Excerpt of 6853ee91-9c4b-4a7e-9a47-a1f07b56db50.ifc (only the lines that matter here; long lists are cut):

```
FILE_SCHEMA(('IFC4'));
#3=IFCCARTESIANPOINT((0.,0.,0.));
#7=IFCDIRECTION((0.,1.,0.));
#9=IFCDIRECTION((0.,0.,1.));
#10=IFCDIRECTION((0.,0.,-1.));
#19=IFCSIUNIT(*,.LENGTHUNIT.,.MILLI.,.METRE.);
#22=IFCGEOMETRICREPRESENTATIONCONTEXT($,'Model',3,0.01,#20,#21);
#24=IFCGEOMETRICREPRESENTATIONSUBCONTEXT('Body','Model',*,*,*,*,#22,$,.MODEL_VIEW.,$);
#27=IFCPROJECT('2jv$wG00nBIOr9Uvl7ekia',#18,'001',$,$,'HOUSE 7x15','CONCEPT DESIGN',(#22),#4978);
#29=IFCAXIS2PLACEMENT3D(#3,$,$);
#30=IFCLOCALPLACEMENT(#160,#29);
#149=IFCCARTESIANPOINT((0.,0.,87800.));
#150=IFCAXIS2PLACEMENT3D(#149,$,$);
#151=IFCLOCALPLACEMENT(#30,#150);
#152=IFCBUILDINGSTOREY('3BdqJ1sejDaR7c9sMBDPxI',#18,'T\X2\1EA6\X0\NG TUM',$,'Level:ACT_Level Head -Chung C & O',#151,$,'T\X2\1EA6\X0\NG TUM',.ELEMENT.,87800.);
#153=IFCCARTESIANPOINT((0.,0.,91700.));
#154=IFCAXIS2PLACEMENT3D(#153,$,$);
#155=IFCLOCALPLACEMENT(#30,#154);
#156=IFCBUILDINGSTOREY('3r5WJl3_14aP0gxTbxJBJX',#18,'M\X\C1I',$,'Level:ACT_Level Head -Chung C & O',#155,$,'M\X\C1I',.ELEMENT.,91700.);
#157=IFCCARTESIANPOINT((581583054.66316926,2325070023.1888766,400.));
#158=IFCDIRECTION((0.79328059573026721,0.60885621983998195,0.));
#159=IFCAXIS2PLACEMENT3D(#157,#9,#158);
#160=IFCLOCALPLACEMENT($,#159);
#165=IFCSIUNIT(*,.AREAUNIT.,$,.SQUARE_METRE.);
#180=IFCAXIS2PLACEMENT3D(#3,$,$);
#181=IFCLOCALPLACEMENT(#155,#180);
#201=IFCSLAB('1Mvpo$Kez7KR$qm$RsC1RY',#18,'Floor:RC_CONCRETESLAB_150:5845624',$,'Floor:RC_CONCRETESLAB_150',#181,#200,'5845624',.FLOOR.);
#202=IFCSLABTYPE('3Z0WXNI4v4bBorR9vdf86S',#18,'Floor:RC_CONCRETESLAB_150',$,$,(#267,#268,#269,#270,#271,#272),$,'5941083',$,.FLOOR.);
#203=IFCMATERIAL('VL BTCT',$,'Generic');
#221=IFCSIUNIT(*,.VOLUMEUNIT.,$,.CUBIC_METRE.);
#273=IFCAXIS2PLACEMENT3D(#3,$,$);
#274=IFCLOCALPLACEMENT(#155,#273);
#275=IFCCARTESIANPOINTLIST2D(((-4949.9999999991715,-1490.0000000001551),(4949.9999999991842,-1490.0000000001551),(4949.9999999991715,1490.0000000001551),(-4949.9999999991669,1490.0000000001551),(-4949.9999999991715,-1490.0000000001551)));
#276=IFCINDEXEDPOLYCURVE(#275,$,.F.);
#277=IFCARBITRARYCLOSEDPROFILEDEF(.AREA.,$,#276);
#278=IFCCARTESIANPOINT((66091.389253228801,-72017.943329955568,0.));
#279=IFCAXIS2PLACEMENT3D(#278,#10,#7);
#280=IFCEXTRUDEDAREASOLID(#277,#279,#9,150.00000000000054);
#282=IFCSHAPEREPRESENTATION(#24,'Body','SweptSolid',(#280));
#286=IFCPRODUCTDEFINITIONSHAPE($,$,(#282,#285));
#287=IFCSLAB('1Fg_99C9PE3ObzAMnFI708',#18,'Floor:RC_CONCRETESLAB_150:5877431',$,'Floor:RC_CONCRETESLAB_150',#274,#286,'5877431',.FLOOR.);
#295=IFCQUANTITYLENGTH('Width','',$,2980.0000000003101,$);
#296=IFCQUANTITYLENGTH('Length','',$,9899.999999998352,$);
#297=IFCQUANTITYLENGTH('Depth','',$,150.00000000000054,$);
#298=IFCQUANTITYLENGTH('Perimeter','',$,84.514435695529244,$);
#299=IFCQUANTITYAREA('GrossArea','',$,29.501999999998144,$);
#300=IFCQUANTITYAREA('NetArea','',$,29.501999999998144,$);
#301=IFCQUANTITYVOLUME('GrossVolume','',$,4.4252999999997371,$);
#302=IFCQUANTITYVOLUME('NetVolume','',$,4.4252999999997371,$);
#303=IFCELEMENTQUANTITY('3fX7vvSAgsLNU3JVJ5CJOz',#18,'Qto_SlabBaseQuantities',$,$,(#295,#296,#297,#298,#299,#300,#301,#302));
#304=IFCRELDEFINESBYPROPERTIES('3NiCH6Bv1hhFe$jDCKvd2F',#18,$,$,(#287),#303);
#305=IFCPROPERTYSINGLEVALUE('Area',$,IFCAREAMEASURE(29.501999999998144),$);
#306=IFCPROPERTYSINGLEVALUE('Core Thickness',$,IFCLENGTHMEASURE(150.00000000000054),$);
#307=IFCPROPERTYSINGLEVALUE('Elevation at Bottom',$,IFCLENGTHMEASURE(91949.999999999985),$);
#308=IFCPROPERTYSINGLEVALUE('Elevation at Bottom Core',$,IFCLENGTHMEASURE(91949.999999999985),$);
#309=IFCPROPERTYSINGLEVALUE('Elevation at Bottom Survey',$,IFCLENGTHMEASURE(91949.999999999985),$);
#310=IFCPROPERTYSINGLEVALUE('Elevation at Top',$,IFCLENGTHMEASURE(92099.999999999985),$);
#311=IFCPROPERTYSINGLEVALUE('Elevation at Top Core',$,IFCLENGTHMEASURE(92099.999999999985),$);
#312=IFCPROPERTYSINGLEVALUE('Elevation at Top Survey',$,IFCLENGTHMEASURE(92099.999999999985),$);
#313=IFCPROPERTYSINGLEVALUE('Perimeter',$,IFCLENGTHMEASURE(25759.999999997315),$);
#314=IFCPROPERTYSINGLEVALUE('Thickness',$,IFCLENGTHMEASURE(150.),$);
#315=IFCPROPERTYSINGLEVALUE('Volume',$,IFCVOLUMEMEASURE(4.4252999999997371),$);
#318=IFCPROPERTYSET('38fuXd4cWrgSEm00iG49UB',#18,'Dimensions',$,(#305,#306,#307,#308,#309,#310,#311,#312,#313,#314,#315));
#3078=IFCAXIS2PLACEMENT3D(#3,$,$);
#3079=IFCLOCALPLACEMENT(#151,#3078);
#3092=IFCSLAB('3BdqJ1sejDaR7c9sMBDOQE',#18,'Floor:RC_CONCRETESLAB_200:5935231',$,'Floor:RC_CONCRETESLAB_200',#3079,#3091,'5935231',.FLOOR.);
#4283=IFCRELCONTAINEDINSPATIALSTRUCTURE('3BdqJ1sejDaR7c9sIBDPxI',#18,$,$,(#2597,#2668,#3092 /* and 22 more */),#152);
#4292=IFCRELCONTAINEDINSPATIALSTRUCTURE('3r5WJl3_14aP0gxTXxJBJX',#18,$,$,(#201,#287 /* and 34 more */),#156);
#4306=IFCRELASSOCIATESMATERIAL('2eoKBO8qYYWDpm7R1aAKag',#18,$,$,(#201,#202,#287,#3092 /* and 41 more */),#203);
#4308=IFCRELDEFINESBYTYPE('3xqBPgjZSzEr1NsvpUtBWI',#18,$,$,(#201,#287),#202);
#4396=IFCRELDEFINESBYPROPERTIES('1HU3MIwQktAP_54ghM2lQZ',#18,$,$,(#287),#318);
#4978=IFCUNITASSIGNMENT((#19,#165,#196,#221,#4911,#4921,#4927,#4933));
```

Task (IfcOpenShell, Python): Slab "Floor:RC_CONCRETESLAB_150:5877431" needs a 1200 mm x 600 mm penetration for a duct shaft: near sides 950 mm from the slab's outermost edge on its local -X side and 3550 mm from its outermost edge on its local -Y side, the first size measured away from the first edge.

```python
import numpy as np
import ifcopenshell
import ifcopenshell.api.feature
import ifcopenshell.api.geometry
import ifcopenshell.api.pset
import ifcopenshell.api.root
import ifcopenshell.geom
import ifcopenshell.util.element
import ifcopenshell.util.placement
import ifcopenshell.util.representation
import ifcopenshell.util.shape
import ifcopenshell.util.unit

model = ifcopenshell.open("6853ee91-9c4b-4a7e-9a47-a1f07b56db50.ifc")
unit_scale = ifcopenshell.util.unit.calculate_unit_scale(model)
area_scale = ifcopenshell.util.unit.calculate_unit_scale(model, "AREAUNIT")
volume_scale = ifcopenshell.util.unit.calculate_unit_scale(model, "VOLUMEUNIT")
settings = ifcopenshell.geom.settings()


def volume(element):
    """Net volume in cubic metres, openings subtracted."""
    shape = ifcopenshell.geom.create_shape(settings, element)
    return ifcopenshell.util.shape.get_volume(shape.geometry)


slab = model.by_guid("1Fg_99C9PE3ObzAMnFI708")
before = volume(slab)

# Extent in the slab's own axes, in metres. The edges named are its -X and -Y sides.
slab_shape = ifcopenshell.geom.create_shape(settings, slab)
vertices = ifcopenshell.util.shape.get_vertices(slab_shape.geometry)
x_min, y_min, bottom = vertices.min(axis=0)
top = vertices[:, 2].max()

opening = ifcopenshell.api.root.create_entity(model, ifc_class="IfcOpeningElement", name="Duct shaft opening", predefined_type="OPENING")
context = ifcopenshell.util.representation.get_context(model, "Model", "Body", "MODEL_VIEW")
width, depth = 1.2, 0.6
outline = [(0.0, 0.0), (width, 0.0), (width, depth), (0.0, depth), (0.0, 0.0)]
# Overshoot both faces by 50 mm so the cut is clean.
shape = ifcopenshell.api.geometry.add_slab_representation(
    model, context=context, depth=top - bottom + 0.1, polyline=outline
)
ifcopenshell.api.geometry.assign_representation(model, product=opening, representation=shape)

matrix = ifcopenshell.util.placement.get_local_placement(slab.ObjectPlacement)
matrix[:, 3] = matrix @ np.append(np.array([x_min + 0.95, y_min + 3.55, bottom - 0.05]) / unit_scale, 1.0)
ifcopenshell.api.geometry.edit_object_placement(model, product=opening, matrix=matrix, is_si=False)
ifcopenshell.api.feature.add_feature(model, feature=opening, element=slab)

after = volume(slab)

# Update the slab's stored quantities.
qto = model.by_id(ifcopenshell.util.element.get_pset(slab, "Qto_SlabBaseQuantities", should_inherit=False)["id"])
ifcopenshell.api.pset.edit_qto(model, qto=qto, properties={
    "NetArea": after / (top - bottom) / area_scale,
    "NetVolume": after / volume_scale,
})
pset = model.by_id(ifcopenshell.util.element.get_pset(slab, "Dimensions", should_inherit=False)["id"])
ifcopenshell.api.pset.edit_pset(model, pset=pset, properties={
    "Area": model.create_entity("IfcAreaMeasure", after / (top - bottom) / area_scale),
    "Volume": model.create_entity("IfcVolumeMeasure", after / volume_scale),
})

print(f"slab volume {before:.3f} -> {after:.3f} m3")

model.write("6853ee91-9c4b-4a7e-9a47-a1f07b56db50_rev.ifc")
```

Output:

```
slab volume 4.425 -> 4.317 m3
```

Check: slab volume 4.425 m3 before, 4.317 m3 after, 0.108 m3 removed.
